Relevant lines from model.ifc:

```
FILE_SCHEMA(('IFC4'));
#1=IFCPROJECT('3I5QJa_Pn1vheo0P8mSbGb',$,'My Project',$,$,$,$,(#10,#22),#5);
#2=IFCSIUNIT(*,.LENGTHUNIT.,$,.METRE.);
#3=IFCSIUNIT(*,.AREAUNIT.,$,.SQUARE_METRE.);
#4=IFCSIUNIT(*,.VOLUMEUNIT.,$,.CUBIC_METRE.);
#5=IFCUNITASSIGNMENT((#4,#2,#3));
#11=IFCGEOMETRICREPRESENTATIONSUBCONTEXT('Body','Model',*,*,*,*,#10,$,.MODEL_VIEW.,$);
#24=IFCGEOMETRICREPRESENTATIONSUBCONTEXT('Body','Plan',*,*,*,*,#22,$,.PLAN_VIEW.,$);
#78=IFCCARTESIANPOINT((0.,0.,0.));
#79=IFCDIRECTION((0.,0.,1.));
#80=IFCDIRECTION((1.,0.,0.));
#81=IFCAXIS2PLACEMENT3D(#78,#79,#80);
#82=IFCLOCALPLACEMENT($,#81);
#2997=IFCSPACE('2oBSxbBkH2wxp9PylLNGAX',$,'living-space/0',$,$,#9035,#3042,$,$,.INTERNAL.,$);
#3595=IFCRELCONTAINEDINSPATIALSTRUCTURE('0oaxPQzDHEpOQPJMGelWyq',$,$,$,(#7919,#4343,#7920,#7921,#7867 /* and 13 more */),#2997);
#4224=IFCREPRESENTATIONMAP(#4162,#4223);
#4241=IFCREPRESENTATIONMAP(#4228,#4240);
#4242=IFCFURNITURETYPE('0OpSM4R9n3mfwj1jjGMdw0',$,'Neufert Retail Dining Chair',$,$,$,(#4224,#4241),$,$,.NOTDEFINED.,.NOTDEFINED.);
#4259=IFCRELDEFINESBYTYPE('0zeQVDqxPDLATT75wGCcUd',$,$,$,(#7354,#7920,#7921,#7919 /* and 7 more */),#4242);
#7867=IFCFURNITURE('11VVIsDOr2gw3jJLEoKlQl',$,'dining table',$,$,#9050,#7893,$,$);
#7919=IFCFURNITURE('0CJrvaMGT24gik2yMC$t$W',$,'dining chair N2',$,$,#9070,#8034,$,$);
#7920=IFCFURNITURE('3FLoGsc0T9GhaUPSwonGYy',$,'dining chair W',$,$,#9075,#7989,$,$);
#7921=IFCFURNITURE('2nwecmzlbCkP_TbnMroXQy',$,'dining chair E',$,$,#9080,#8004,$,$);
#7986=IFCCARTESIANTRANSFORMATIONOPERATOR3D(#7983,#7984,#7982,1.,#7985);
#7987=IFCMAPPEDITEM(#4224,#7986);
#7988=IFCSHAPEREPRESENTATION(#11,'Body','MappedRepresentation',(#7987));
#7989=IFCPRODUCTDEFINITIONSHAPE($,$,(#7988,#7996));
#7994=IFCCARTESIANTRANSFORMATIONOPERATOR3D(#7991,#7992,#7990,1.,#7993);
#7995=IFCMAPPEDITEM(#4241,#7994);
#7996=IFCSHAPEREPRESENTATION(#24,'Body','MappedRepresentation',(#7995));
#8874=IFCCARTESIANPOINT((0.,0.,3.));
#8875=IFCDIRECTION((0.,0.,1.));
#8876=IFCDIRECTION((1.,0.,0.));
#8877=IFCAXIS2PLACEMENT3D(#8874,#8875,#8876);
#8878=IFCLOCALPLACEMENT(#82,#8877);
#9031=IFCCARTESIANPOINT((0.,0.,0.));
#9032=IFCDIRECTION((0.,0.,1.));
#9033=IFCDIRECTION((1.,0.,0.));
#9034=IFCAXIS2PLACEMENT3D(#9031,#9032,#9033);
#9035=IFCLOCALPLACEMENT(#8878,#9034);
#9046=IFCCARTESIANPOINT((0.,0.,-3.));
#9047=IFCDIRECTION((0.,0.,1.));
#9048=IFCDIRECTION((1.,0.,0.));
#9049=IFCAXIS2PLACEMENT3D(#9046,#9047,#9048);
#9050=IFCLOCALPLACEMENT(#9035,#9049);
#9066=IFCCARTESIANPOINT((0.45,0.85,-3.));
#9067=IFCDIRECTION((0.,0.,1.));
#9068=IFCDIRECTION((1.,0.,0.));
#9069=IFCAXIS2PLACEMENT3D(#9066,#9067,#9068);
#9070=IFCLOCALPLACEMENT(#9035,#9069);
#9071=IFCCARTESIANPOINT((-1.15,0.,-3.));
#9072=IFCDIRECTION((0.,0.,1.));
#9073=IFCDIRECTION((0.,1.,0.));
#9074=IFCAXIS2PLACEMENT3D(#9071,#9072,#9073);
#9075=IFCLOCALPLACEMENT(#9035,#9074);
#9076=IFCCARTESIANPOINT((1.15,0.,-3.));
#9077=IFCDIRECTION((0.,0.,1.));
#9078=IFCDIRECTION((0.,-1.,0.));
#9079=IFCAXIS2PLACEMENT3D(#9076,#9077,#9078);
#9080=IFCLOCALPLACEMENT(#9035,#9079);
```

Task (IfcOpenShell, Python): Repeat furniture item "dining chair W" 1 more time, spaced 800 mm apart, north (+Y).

```python
import numpy as np
import ifcopenshell
import ifcopenshell.api.geometry
import ifcopenshell.api.root
import ifcopenshell.util.element
import ifcopenshell.util.placement
import ifcopenshell.util.unit

model = ifcopenshell.open("model.ifc")
unit_scale = ifcopenshell.util.unit.calculate_unit_scale(model)

source = model.by_id(7920)
base = ifcopenshell.util.placement.get_local_placement(source.ObjectPlacement)
step = np.array([0.0, 1.0, 0.0]) * 0.8 / unit_scale

for i in range(1, 2):
    copy = ifcopenshell.api.root.copy_class(model, product=source)
    copy.Representation = ifcopenshell.util.element.copy_deep(
        model, source.Representation, exclude=["IfcGeometricRepresentationContext", "IfcRepresentationMap"]
    )
    matrix = base.copy()
    matrix[:3, 3] += i * step
    print("added at", matrix[:3, 3].round(3) + 0.0)
    ifcopenshell.api.geometry.edit_object_placement(model, product=copy, matrix=matrix, is_si=False)

model.write("model_edited.ifc")
```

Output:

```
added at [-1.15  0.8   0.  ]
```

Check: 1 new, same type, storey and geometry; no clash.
